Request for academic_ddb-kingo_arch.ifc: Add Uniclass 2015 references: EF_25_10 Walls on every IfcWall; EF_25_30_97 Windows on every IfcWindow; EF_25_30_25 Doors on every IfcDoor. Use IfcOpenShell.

First a look at what the model holds.

```python
import ifcopenshell

model = ifcopenshell.open("academic_ddb-kingo_arch.ifc")
print(model.schema)
print("classifications:", [c.Name for c in model.by_type("IfcClassification")])
for ifc_class in ("IfcDoor", "IfcRoof", "IfcStair", "IfcWall", "IfcWindow"):
    print(ifc_class, len(model.by_type(ifc_class)))
```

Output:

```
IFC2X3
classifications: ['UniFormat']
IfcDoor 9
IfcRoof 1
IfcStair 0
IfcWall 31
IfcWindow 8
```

```python
import ifcopenshell
import ifcopenshell.api.classification

model = ifcopenshell.open("academic_ddb-kingo_arch.ifc")

# IFC2X3 requires Source and Edition and has no link from the project to the system.
system = model.create_entity("IfcClassification", Source="NBS", Edition="2015", Name="Uniclass 2015")

codes = {
    "IfcWall": ("EF_25_10", "Walls"),
    "IfcWindow": ("EF_25_30_97", "Windows"),
    "IfcDoor": ("EF_25_30_25", "Doors"),
}
for ifc_class, (code, name) in codes.items():
    products = model.by_type(ifc_class)
    ifcopenshell.api.classification.add_reference(
        model, products=products, classification=system, identification=code, name=name
    )
    print(code, len(products))

model.write("academic_ddb-kingo_arch_edited.ifc")
```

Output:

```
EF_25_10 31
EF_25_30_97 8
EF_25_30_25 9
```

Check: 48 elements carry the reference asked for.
